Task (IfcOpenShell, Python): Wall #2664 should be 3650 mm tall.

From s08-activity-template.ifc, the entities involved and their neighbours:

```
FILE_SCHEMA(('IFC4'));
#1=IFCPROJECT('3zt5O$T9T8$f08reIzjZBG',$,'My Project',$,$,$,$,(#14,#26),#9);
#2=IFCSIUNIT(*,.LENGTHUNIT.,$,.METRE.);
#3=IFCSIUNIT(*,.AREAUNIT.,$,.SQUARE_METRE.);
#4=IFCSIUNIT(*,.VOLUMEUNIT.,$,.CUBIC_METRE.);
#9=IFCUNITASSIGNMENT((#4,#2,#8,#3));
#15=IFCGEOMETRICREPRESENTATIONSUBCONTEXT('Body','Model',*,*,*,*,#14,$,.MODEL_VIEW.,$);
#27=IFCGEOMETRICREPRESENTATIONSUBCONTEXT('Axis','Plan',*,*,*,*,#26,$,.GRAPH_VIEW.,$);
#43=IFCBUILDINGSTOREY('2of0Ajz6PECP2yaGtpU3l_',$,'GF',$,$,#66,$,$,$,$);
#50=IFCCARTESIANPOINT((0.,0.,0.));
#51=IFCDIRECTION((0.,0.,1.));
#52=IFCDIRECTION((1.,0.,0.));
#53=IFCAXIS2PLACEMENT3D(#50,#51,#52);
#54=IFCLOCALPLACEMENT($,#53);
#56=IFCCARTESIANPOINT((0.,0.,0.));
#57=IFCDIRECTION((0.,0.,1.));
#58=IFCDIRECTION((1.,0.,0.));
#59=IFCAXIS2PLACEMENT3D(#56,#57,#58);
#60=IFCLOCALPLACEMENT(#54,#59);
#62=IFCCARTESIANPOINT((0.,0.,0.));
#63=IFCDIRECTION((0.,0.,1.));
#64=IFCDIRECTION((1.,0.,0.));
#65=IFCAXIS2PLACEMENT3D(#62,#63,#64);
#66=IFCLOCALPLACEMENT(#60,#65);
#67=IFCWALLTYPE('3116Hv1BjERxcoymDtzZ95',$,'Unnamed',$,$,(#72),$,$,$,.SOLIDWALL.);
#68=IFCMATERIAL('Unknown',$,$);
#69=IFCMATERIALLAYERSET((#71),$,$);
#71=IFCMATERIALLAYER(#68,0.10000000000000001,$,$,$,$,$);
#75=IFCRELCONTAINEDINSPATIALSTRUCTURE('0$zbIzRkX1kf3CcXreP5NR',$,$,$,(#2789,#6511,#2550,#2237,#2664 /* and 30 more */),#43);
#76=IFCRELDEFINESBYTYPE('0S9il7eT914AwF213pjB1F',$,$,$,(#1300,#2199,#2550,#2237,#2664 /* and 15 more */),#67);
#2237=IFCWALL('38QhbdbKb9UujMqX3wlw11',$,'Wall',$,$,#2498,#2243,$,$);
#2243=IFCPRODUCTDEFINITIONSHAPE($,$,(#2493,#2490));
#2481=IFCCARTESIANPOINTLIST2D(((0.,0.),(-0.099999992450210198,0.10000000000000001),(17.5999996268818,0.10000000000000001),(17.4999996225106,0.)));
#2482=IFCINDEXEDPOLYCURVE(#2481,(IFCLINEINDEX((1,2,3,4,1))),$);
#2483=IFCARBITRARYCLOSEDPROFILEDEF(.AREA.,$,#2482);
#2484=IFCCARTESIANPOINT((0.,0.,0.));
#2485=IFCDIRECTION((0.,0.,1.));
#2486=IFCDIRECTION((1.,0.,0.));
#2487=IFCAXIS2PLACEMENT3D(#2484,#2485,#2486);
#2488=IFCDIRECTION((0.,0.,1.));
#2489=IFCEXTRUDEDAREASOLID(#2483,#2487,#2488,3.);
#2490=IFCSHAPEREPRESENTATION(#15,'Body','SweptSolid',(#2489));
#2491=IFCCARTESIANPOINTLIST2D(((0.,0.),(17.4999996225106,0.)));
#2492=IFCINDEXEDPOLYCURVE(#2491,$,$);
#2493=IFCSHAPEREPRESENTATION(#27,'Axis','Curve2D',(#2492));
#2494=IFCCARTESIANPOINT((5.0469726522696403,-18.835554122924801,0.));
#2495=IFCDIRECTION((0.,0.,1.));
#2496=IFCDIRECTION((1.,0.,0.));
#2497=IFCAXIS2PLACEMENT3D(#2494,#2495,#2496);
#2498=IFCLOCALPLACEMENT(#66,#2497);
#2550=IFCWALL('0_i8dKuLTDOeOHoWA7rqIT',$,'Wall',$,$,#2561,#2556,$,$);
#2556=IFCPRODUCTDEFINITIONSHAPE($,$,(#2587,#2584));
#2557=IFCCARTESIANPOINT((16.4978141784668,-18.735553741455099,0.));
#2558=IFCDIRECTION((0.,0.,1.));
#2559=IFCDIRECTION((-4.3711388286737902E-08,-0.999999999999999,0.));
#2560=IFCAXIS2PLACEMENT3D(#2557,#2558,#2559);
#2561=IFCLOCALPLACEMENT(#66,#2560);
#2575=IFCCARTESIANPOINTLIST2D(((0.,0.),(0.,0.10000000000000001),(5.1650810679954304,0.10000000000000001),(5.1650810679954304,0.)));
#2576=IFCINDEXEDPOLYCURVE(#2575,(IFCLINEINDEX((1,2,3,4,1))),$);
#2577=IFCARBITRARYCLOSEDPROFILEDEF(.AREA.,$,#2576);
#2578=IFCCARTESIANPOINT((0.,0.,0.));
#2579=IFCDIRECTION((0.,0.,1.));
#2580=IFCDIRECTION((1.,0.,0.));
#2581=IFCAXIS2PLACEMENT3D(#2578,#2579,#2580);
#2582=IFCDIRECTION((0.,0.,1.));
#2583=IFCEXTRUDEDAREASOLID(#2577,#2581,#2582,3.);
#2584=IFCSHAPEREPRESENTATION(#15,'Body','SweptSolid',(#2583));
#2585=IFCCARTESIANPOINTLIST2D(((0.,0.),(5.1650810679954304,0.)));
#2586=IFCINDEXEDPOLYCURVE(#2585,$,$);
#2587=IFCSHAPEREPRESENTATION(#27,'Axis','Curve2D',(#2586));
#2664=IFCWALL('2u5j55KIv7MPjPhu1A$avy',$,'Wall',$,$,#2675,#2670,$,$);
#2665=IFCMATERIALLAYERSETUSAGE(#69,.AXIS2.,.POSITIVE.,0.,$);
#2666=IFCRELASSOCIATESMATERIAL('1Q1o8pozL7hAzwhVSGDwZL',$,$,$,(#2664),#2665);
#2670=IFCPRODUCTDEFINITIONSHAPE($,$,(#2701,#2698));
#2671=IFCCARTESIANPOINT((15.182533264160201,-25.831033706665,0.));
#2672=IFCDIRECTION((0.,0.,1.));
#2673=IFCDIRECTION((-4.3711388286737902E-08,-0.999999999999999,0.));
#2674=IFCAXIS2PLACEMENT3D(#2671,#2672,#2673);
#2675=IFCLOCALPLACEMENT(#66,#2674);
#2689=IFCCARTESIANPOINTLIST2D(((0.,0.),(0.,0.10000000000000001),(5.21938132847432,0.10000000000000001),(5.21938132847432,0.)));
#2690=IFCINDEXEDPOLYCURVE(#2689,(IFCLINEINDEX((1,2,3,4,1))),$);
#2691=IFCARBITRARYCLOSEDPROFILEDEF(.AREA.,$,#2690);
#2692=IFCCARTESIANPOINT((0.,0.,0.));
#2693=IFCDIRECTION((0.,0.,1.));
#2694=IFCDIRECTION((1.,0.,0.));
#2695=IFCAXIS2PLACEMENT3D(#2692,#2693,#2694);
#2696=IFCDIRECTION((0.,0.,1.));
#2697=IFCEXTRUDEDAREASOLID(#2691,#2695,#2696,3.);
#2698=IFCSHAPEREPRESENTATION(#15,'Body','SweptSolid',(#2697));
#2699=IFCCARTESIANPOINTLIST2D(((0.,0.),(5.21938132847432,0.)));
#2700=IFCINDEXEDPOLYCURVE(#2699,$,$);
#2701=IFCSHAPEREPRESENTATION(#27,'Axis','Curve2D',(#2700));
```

```python
import ifcopenshell
import ifcopenshell.geom
import ifcopenshell.util.representation
import ifcopenshell.util.shape
import ifcopenshell.util.unit

model = ifcopenshell.open("s08-activity-template.ifc")
unit_scale = ifcopenshell.util.unit.calculate_unit_scale(model)
settings = ifcopenshell.geom.settings()


def volume(element):
    """Net volume in cubic metres, openings subtracted."""
    shape = ifcopenshell.geom.create_shape(settings, element)
    return ifcopenshell.util.shape.get_volume(shape.geometry)


wall = model.by_guid("2u5j55KIv7MPjPhu1A$avy")
before = volume(wall)

body = ifcopenshell.util.representation.get_representation(wall, "Model", "Body")
solid = body.Items[0]
old_height = solid.Depth
solid.Depth = 3.65 / unit_scale
after = volume(wall)

print(f"height {old_height:g} -> {solid.Depth:g}, volume {before:.3f} -> {after:.3f} m3")

model.write("s08-activity-template-out.ifc")
```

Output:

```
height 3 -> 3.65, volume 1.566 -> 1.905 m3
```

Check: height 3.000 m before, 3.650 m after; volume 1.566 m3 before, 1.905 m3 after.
